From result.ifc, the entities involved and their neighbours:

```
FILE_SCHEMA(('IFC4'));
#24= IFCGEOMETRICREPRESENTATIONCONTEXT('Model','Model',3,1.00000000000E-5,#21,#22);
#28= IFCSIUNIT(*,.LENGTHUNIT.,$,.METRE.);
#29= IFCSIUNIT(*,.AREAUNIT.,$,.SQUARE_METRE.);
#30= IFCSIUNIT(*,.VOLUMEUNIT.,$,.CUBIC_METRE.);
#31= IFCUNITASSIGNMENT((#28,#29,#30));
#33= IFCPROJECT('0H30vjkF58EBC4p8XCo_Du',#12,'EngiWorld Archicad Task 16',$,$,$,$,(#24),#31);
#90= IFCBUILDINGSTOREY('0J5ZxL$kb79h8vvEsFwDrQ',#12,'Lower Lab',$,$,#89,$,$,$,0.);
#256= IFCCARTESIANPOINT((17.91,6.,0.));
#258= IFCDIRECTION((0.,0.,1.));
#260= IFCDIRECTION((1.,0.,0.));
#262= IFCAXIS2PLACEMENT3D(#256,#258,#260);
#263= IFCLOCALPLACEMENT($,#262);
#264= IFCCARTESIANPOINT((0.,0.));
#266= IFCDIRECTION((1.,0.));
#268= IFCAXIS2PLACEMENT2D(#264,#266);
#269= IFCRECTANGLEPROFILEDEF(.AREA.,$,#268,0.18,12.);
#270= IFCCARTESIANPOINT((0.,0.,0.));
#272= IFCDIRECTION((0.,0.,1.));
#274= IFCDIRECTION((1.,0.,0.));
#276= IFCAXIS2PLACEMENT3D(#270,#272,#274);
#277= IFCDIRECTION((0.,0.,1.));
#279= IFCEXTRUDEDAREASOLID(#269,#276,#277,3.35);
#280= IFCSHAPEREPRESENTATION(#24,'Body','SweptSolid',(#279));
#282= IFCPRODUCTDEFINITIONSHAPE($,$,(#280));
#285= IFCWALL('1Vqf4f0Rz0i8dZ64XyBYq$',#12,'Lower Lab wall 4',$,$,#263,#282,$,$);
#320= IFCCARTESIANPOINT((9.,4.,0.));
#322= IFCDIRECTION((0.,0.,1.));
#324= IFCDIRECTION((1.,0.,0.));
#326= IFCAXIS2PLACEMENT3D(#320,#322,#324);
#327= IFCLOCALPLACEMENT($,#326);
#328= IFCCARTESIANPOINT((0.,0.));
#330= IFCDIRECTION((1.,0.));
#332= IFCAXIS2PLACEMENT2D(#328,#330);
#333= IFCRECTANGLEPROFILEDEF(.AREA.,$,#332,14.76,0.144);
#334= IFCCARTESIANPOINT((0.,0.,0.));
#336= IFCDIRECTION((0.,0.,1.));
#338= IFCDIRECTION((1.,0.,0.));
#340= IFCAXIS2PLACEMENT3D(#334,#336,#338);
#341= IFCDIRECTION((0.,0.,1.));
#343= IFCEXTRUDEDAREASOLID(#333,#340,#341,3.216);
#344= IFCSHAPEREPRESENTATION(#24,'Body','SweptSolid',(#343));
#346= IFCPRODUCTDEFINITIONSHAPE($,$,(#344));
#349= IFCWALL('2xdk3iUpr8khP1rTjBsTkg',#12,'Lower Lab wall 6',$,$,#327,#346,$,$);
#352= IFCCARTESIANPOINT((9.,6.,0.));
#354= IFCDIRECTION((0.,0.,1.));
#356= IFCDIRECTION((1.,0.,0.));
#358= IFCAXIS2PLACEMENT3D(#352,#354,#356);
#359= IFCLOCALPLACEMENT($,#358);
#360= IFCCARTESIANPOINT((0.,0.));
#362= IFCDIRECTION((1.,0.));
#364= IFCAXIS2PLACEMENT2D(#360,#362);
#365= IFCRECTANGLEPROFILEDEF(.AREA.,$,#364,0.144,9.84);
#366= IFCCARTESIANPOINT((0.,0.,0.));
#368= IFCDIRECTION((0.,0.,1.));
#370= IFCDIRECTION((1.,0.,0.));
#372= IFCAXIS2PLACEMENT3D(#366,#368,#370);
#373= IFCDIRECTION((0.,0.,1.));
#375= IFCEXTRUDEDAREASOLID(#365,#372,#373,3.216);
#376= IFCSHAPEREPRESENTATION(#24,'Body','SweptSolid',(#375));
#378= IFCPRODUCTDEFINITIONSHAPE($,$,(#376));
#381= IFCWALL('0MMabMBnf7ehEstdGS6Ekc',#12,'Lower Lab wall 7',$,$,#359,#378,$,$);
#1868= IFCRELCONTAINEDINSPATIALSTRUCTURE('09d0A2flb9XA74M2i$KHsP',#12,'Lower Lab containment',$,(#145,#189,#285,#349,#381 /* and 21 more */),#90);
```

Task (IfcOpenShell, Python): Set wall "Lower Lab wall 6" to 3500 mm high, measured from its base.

```python
import ifcopenshell
import ifcopenshell.geom
import ifcopenshell.util.shape

model = ifcopenshell.open("result.ifc")
settings = ifcopenshell.geom.settings()


def volume(element):
    """Net volume in cubic metres, openings subtracted."""
    shape = ifcopenshell.geom.create_shape(settings, element)
    return ifcopenshell.util.shape.get_volume(shape.geometry)


wall = model.by_guid("2xdk3iUpr8khP1rTjBsTkg")
before = volume(wall)

body = next(r for r in wall.Representation.Representations if r.RepresentationIdentifier == "Body")
solid = body.Items[0]
old_height = solid.Depth
solid.Depth = 3.5
after = volume(wall)

print(f"height {old_height:g} -> {solid.Depth:g}, volume {before:.3f} -> {after:.3f} m3")

model.write("result_edited.ifc")
```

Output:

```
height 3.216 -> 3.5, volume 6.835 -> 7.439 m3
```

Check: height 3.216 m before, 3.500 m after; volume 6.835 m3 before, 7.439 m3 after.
